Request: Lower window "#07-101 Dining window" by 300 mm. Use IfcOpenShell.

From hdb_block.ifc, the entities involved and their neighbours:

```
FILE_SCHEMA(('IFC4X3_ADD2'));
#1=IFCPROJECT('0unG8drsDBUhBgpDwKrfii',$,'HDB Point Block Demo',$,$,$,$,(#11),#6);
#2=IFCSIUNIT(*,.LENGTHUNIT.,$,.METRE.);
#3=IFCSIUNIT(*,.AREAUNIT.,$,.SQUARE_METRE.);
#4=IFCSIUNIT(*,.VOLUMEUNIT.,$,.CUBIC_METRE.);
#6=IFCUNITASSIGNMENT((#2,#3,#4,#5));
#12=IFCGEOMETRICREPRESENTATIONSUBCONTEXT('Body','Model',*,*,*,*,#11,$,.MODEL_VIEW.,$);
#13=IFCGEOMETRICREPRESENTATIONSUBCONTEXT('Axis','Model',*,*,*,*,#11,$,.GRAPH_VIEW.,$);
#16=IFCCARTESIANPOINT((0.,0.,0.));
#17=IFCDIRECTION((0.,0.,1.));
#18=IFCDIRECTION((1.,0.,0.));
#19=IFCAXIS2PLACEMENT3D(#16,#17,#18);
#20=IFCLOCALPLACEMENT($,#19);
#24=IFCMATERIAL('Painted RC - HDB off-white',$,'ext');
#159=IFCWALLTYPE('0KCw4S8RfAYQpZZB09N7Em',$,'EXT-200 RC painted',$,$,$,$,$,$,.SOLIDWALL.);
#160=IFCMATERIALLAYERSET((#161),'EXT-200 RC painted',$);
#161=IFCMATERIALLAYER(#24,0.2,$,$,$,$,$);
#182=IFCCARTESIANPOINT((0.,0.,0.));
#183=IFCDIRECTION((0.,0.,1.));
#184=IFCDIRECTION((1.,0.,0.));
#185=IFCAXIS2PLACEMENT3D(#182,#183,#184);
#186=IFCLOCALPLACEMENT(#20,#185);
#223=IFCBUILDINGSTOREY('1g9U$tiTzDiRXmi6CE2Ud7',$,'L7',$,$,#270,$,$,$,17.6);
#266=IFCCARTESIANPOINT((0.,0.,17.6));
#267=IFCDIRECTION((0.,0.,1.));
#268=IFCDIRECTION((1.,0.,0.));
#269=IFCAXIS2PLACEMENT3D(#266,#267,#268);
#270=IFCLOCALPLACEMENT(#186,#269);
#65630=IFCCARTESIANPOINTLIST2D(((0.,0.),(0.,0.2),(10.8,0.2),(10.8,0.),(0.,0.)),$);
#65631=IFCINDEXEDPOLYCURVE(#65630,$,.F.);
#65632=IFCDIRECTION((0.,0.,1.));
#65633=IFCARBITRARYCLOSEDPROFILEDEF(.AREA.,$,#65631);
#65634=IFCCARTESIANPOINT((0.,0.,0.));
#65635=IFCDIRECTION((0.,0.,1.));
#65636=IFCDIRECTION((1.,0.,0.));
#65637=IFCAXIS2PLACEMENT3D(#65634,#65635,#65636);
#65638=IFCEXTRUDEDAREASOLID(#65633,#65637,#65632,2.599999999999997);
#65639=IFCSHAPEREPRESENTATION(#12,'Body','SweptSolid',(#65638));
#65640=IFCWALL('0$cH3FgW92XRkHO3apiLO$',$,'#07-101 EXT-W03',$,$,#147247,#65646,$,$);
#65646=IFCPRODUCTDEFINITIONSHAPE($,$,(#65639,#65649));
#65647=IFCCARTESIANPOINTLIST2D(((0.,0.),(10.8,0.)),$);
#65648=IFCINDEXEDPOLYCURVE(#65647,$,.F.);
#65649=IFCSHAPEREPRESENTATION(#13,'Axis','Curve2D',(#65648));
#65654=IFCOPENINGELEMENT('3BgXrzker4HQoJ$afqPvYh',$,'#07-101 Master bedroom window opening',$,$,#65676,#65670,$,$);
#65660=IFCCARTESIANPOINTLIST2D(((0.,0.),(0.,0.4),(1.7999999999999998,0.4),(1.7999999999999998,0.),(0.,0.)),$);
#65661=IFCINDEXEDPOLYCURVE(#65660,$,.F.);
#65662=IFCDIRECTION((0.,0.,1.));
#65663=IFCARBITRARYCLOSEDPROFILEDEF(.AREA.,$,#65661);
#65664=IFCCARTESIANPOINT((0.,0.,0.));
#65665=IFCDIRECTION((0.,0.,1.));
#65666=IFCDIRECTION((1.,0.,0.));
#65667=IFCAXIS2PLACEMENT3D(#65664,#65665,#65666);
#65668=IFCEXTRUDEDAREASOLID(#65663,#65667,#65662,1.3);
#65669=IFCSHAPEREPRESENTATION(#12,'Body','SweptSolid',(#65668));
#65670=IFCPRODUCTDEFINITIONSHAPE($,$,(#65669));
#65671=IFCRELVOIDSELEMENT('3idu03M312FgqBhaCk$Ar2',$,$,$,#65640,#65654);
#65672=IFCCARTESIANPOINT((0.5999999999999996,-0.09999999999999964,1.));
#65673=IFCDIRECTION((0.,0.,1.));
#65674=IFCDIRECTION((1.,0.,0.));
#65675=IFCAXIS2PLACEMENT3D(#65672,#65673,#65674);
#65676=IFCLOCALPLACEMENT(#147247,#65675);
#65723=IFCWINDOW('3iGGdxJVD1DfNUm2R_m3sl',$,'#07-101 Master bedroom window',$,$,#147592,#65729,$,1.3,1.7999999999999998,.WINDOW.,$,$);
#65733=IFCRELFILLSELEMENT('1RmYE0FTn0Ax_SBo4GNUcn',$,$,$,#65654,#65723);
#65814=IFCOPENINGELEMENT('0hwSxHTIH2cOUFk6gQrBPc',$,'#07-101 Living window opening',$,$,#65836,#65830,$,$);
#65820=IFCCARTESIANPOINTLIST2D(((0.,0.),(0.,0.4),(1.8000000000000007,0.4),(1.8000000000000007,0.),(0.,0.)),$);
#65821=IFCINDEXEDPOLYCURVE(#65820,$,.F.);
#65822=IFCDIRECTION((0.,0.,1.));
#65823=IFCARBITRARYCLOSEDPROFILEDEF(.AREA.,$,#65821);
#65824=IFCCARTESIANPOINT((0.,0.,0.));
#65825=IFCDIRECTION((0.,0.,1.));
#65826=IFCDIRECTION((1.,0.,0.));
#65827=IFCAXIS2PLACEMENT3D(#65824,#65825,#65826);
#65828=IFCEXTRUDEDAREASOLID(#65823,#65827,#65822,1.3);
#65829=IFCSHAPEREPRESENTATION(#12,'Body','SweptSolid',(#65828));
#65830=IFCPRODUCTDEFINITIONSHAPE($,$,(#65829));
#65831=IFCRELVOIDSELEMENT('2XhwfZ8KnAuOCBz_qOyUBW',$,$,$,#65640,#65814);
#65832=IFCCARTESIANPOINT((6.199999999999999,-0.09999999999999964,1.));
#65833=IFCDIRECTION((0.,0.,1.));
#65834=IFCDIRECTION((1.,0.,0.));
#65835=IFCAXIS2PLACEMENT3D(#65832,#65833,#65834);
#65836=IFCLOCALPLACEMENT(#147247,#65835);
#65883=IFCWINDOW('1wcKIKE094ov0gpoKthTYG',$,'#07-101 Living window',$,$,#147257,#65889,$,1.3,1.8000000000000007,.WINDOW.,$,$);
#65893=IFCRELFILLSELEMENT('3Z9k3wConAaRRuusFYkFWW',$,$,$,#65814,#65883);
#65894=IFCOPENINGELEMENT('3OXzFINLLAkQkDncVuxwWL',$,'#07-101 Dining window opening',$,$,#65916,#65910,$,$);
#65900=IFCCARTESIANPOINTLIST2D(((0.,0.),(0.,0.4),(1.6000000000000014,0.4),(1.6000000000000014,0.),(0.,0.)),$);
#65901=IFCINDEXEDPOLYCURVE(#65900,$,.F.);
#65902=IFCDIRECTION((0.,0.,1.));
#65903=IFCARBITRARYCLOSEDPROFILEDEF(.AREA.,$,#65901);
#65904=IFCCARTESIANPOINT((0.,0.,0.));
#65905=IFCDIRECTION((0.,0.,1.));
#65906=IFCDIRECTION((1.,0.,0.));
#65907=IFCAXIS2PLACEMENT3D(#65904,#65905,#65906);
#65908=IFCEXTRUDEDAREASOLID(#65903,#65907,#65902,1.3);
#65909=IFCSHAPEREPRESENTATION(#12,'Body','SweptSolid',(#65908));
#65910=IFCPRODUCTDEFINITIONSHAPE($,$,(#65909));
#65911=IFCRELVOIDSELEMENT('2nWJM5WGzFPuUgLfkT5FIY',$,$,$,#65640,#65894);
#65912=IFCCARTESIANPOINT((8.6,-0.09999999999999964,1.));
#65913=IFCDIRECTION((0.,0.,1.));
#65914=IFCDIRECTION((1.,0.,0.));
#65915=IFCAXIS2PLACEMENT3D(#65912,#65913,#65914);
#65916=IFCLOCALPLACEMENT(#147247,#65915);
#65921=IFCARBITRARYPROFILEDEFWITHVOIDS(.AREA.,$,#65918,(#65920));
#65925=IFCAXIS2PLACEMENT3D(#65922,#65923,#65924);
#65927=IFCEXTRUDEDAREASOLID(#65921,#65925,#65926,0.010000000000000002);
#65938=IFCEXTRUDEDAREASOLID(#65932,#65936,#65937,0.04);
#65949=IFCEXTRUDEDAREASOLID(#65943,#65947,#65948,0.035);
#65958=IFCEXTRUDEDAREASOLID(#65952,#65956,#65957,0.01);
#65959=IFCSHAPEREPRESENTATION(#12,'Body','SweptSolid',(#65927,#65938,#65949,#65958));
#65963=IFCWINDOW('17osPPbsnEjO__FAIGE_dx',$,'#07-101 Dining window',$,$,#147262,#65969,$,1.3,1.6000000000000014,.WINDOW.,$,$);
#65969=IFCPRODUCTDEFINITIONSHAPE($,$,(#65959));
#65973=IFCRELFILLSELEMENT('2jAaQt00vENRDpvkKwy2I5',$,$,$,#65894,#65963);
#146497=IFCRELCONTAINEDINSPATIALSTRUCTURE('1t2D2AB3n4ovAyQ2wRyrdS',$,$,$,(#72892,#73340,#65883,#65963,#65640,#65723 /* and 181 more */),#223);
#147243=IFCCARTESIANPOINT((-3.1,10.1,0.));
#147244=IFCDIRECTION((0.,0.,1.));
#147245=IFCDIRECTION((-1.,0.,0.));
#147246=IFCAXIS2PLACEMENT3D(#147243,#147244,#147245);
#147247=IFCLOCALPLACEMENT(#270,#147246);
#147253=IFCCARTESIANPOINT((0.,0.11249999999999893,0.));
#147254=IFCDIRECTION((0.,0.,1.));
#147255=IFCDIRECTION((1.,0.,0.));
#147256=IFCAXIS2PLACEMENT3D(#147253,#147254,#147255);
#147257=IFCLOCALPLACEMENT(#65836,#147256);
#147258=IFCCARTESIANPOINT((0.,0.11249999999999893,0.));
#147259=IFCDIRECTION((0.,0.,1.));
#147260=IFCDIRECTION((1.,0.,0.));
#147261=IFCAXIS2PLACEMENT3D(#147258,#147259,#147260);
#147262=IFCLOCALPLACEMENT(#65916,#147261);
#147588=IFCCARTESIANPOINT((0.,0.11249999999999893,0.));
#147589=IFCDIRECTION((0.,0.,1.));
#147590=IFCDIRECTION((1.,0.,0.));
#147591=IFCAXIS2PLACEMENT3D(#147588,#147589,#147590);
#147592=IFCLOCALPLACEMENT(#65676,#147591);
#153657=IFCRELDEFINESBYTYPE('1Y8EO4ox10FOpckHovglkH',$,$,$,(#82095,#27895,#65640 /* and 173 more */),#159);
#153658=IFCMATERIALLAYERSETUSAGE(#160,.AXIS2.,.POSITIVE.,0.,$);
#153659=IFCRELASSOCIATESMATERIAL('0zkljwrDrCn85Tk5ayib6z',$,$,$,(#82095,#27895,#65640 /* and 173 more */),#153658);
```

```python
import numpy as np
import ifcopenshell
import ifcopenshell.api.geometry
import ifcopenshell.util.placement
import ifcopenshell.util.unit

model = ifcopenshell.open("hdb_block.ifc")
unit_scale = ifcopenshell.util.unit.calculate_unit_scale(model)

window = model.by_guid("17osPPbsnEjO__FAIGE_dx")
opening = window.FillsVoids[0].RelatingOpeningElement
dz = -0.3 / unit_scale

shift = np.array([0.0, 0.0, dz])
# The window is placed relative to its opening, so it follows when the opening moves.
matrix = ifcopenshell.util.placement.get_local_placement(opening.ObjectPlacement)
matrix[:3, 3] += shift
ifcopenshell.api.geometry.edit_object_placement(
    model, product=opening, matrix=matrix, is_si=False, should_transform_children=True
)

print(f"moved by {dz * unit_scale:+.3f} m")

model.write("hdb_block-out.ifc")
```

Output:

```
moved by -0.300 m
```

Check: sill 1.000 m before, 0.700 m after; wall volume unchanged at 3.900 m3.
